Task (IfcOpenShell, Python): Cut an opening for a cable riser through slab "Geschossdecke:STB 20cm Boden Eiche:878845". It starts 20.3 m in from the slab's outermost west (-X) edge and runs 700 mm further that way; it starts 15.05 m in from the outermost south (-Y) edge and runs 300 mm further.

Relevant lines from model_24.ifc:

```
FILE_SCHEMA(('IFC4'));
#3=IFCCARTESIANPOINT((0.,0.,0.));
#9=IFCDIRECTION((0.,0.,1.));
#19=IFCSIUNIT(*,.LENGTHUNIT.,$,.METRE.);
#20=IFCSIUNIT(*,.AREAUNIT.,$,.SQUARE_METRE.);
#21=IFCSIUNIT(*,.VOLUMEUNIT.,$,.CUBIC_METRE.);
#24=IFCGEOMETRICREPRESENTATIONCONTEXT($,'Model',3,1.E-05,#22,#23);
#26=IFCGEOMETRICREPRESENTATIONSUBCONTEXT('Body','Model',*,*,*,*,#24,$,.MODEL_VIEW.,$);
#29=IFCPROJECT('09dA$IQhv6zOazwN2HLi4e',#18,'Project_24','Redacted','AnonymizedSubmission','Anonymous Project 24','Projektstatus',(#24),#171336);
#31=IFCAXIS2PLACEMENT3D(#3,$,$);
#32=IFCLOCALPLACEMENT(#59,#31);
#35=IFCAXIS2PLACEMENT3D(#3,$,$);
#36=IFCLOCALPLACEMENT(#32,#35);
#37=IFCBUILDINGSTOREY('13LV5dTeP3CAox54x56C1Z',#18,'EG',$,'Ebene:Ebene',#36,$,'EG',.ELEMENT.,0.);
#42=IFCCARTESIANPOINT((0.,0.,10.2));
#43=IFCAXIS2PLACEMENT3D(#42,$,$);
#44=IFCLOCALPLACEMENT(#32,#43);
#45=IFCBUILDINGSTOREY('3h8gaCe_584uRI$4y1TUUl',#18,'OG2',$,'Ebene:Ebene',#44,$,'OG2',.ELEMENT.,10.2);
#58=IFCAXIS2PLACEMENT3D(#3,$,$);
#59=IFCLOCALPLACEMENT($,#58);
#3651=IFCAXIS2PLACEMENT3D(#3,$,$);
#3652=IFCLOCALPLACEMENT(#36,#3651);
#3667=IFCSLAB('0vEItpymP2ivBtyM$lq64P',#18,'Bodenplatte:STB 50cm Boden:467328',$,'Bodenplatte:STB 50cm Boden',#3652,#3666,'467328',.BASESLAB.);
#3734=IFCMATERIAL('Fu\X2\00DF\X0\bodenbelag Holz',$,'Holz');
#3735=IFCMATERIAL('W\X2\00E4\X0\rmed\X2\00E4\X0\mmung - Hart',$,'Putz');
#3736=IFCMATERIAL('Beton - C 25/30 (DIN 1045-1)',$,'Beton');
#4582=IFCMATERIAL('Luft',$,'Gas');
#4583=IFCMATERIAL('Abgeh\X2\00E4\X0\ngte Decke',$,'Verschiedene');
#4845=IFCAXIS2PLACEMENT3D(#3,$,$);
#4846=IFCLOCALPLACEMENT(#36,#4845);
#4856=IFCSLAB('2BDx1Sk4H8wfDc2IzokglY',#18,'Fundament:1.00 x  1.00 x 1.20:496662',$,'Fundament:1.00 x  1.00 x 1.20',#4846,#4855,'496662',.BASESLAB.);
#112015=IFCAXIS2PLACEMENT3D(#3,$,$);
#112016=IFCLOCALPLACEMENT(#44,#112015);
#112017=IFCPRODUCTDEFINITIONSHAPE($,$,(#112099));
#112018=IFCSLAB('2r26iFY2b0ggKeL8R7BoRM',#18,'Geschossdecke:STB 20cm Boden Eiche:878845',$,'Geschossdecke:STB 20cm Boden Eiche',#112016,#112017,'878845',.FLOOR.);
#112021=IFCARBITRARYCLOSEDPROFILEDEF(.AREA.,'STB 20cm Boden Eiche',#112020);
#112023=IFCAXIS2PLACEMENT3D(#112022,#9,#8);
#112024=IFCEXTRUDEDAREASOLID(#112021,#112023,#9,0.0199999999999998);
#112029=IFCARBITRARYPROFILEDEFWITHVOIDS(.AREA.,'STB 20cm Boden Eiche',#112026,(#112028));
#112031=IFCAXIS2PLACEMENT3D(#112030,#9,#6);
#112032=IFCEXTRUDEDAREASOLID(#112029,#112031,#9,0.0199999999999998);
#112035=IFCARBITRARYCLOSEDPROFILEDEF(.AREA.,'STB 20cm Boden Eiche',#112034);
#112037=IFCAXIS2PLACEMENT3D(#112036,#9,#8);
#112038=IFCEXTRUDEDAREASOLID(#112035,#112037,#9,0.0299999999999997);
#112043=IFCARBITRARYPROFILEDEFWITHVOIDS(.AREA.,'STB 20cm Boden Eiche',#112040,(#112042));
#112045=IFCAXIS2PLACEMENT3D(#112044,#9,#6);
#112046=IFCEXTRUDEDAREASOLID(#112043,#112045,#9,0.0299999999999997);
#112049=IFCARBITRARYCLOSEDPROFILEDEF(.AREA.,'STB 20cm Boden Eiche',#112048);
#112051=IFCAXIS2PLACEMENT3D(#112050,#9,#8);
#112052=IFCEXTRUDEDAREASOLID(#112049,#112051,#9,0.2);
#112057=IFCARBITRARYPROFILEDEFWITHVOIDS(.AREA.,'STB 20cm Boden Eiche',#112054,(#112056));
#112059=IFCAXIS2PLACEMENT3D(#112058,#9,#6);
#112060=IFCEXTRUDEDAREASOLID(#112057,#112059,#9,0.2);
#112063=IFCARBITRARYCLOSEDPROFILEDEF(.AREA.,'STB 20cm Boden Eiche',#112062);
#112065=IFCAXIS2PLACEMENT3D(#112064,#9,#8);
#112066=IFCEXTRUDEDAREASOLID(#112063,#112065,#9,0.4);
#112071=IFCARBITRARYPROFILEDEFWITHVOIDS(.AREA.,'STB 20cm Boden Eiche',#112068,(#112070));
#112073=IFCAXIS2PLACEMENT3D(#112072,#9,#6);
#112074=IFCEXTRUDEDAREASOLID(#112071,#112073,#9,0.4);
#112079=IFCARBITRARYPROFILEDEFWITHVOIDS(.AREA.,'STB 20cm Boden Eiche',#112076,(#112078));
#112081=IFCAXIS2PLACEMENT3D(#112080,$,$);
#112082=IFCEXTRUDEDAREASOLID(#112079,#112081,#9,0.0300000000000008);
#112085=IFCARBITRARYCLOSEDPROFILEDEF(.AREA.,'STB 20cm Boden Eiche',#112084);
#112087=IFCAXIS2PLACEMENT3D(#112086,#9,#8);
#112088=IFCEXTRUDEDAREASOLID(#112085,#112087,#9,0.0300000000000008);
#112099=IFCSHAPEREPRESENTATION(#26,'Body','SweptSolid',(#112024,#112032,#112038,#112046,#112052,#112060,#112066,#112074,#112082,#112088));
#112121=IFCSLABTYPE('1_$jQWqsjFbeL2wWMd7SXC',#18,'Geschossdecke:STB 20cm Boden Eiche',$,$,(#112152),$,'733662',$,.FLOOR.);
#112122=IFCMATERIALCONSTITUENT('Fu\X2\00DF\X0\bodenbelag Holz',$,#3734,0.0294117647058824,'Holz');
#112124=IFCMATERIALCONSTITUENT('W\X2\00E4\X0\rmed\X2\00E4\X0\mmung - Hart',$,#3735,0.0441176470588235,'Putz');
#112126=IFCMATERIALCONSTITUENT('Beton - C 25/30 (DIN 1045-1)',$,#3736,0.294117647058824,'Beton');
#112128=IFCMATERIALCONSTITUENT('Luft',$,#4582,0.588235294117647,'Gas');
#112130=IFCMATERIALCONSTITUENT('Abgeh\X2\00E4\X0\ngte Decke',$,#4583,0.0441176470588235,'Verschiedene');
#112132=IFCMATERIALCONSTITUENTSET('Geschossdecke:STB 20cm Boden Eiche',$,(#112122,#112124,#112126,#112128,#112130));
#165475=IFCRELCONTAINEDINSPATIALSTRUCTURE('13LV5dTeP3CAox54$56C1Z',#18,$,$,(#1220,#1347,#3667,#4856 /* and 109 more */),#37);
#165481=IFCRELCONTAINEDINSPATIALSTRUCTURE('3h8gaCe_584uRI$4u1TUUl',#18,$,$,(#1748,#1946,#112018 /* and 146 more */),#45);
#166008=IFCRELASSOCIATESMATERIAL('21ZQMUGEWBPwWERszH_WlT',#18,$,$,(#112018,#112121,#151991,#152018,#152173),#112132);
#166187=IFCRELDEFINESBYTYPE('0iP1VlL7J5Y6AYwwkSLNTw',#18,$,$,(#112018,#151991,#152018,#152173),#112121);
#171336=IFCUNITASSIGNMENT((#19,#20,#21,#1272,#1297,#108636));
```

```python
import numpy as np
import ifcopenshell
import ifcopenshell.api.feature
import ifcopenshell.api.geometry
import ifcopenshell.api.root
import ifcopenshell.geom
import ifcopenshell.util.placement
import ifcopenshell.util.representation
import ifcopenshell.util.shape
import ifcopenshell.util.unit

model = ifcopenshell.open("model_24.ifc")
unit_scale = ifcopenshell.util.unit.calculate_unit_scale(model)
settings = ifcopenshell.geom.settings()


def volume(element):
    """Net volume in cubic metres, openings subtracted."""
    shape = ifcopenshell.geom.create_shape(settings, element)
    return ifcopenshell.util.shape.get_volume(shape.geometry)


slab = model.by_id(112018)
before = volume(slab)

# Extent in the slab's own axes, in metres. The edges named are its -X and -Y sides.
slab_shape = ifcopenshell.geom.create_shape(settings, slab)
vertices = ifcopenshell.util.shape.get_vertices(slab_shape.geometry)
x_min, y_min, bottom = vertices.min(axis=0)
top = vertices[:, 2].max()

opening = ifcopenshell.api.root.create_entity(model, ifc_class="IfcOpeningElement", name="Cable riser opening", predefined_type="OPENING")
context = ifcopenshell.util.representation.get_context(model, "Model", "Body", "MODEL_VIEW")
width, depth = 0.7, 0.3
outline = [(0.0, 0.0), (width, 0.0), (width, depth), (0.0, depth), (0.0, 0.0)]
# Overshoot both faces by 50 mm so the cut is clean.
shape = ifcopenshell.api.geometry.add_slab_representation(
    model, context=context, depth=top - bottom + 0.1, polyline=outline
)
ifcopenshell.api.geometry.assign_representation(model, product=opening, representation=shape)

matrix = ifcopenshell.util.placement.get_local_placement(slab.ObjectPlacement)
matrix[:, 3] = matrix @ np.append(np.array([x_min + 20.3, y_min + 15.05, bottom - 0.05]) / unit_scale, 1.0)
ifcopenshell.api.geometry.edit_object_placement(model, product=opening, matrix=matrix, is_si=False)
ifcopenshell.api.feature.add_feature(model, feature=opening, element=slab)

after = volume(slab)

print(f"slab volume {before:.3f} -> {after:.3f} m3")

model.write("model_24-out.ifc")
```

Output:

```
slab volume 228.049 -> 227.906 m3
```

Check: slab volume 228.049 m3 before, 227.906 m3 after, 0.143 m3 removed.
